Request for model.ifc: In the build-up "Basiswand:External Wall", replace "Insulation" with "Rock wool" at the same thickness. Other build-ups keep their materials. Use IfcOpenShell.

First a look at what the model holds.

```python
import ifcopenshell
import ifcopenshell.util.element

model = ifcopenshell.open("model.ifc")
print(model.schema)
for layer_set in model.by_type("IfcMaterialLayerSet"):
    if layer_set.LayerSetName == "Basiswand:External Wall":
        for layer in layer_set.MaterialLayers:
            print(layer.id(), layer.Material and layer.Material.Name, layer.LayerThickness, sep=" | ")
        print(len(ifcopenshell.util.element.get_elements_by_material(model, layer_set)), "elements and types use it")
print(sorted(m.Name for m in model.by_type("IfcMaterial") if m.Name)[:60])
```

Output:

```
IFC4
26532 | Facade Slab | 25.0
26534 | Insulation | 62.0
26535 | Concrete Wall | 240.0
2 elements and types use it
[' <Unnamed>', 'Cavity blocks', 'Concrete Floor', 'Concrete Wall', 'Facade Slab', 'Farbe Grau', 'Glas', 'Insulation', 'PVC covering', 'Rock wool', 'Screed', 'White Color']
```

```python
import ifcopenshell
import ifcopenshell.api.material

model = ifcopenshell.open("model.ifc")

layer_set = next(s for s in model.by_type("IfcMaterialLayerSet") if s.LayerSetName == "Basiswand:External Wall")
layer = next(l for l in layer_set.MaterialLayers if l.Material and l.Material.Name == "Insulation")
material = next(m for m in model.by_type("IfcMaterial") if m.Name == "Rock wool")

# Point this one layer at the other material; renaming the old one would change it everywhere.
ifcopenshell.api.material.edit_layer(model, layer=layer, attributes={}, material=material)

print([l.Material.Name if l.Material else None for l in layer_set.MaterialLayers])

model.write("model_v2.ifc")
```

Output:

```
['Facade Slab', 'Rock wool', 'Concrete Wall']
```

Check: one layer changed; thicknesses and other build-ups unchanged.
